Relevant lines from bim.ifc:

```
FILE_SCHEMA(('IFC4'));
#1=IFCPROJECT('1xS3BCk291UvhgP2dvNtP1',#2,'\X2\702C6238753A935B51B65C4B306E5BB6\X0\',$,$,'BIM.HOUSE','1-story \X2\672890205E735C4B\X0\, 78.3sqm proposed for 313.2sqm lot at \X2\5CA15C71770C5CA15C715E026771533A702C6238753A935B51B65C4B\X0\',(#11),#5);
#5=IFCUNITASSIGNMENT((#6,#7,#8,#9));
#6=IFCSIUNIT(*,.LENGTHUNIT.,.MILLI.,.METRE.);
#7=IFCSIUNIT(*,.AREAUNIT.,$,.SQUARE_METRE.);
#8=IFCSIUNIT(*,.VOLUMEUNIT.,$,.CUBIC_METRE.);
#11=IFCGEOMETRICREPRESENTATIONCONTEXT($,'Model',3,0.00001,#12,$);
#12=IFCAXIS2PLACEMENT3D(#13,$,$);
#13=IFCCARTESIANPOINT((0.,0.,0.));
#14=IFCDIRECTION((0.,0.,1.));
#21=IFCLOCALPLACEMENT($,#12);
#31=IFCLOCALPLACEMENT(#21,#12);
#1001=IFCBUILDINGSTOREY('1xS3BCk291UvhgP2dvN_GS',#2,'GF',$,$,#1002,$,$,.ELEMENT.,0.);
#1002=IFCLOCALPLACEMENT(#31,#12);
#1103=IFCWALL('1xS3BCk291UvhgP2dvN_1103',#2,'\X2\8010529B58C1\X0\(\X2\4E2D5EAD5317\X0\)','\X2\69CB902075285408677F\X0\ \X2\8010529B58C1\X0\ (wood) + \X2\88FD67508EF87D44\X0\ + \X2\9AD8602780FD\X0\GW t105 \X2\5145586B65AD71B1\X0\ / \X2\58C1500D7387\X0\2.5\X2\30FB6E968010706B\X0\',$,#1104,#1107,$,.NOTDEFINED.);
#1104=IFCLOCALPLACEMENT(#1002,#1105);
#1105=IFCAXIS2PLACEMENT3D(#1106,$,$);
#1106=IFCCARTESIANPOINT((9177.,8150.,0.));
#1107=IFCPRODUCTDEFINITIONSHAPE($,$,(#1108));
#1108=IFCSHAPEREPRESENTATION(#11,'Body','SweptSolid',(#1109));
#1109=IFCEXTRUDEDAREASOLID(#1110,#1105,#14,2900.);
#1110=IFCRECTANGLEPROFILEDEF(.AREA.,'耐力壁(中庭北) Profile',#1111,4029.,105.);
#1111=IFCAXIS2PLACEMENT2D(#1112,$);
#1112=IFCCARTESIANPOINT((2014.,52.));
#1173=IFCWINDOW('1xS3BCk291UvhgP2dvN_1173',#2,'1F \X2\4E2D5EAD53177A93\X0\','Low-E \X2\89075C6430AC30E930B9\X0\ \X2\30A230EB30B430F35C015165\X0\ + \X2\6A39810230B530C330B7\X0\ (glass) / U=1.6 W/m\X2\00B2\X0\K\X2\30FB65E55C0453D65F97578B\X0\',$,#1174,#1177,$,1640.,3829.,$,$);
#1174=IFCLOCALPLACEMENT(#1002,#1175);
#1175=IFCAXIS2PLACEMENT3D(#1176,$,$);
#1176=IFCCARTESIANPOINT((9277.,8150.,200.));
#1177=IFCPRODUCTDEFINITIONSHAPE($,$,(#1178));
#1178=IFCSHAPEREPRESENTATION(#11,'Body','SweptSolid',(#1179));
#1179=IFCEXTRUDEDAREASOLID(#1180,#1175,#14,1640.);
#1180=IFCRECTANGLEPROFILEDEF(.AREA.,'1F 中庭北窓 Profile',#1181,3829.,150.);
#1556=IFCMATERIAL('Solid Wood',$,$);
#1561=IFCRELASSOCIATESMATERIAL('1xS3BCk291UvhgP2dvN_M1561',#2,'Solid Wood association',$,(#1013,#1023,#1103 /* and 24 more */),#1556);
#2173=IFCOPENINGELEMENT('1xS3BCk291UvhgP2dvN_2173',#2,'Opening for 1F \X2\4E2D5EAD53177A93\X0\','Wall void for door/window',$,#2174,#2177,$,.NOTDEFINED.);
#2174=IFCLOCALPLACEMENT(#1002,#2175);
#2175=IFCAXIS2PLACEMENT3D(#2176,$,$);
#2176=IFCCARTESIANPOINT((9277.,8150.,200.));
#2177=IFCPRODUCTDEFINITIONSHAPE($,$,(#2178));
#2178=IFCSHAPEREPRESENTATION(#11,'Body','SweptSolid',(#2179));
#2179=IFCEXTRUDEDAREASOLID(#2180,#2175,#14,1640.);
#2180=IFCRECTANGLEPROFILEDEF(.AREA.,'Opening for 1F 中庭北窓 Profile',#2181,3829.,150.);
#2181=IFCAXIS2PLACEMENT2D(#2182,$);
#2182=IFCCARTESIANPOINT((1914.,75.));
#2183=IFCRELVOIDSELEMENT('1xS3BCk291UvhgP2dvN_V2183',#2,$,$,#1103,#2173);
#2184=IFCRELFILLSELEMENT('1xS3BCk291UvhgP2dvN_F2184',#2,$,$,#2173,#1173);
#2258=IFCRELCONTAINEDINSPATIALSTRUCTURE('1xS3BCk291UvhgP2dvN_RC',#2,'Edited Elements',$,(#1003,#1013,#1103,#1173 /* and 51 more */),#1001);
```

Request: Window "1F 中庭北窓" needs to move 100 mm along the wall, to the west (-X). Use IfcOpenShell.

```python
import ifcopenshell
import ifcopenshell.api.geometry
import ifcopenshell.util.placement

model = ifcopenshell.open("bim.ifc")

window = model.by_guid("1xS3BCk291UvhgP2dvN_1173")
opening = window.FillsVoids[0].RelatingOpeningElement
wall = opening.VoidsElements[0].RelatingBuildingElement

wall_matrix = ifcopenshell.util.placement.get_local_placement(wall.ObjectPlacement)
shift = wall_matrix[:3, 0] * -100.0
before = ifcopenshell.util.placement.get_local_placement(window.ObjectPlacement)[:3, 3].copy()

# The window is not placed relative to its opening, so move both.
for product in (opening, window):
    matrix = ifcopenshell.util.placement.get_local_placement(product.ObjectPlacement)
    matrix[:3, 3] += shift
    ifcopenshell.api.geometry.edit_object_placement(model, product=product, matrix=matrix, is_si=False)

after = ifcopenshell.util.placement.get_local_placement(window.ObjectPlacement)[:3, 3]
print("window moved by", (after - before).round(3) + 0.0)

model.write("bim_rev.ifc")
```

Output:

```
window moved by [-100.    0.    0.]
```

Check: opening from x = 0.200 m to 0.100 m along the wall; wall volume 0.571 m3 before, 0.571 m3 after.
